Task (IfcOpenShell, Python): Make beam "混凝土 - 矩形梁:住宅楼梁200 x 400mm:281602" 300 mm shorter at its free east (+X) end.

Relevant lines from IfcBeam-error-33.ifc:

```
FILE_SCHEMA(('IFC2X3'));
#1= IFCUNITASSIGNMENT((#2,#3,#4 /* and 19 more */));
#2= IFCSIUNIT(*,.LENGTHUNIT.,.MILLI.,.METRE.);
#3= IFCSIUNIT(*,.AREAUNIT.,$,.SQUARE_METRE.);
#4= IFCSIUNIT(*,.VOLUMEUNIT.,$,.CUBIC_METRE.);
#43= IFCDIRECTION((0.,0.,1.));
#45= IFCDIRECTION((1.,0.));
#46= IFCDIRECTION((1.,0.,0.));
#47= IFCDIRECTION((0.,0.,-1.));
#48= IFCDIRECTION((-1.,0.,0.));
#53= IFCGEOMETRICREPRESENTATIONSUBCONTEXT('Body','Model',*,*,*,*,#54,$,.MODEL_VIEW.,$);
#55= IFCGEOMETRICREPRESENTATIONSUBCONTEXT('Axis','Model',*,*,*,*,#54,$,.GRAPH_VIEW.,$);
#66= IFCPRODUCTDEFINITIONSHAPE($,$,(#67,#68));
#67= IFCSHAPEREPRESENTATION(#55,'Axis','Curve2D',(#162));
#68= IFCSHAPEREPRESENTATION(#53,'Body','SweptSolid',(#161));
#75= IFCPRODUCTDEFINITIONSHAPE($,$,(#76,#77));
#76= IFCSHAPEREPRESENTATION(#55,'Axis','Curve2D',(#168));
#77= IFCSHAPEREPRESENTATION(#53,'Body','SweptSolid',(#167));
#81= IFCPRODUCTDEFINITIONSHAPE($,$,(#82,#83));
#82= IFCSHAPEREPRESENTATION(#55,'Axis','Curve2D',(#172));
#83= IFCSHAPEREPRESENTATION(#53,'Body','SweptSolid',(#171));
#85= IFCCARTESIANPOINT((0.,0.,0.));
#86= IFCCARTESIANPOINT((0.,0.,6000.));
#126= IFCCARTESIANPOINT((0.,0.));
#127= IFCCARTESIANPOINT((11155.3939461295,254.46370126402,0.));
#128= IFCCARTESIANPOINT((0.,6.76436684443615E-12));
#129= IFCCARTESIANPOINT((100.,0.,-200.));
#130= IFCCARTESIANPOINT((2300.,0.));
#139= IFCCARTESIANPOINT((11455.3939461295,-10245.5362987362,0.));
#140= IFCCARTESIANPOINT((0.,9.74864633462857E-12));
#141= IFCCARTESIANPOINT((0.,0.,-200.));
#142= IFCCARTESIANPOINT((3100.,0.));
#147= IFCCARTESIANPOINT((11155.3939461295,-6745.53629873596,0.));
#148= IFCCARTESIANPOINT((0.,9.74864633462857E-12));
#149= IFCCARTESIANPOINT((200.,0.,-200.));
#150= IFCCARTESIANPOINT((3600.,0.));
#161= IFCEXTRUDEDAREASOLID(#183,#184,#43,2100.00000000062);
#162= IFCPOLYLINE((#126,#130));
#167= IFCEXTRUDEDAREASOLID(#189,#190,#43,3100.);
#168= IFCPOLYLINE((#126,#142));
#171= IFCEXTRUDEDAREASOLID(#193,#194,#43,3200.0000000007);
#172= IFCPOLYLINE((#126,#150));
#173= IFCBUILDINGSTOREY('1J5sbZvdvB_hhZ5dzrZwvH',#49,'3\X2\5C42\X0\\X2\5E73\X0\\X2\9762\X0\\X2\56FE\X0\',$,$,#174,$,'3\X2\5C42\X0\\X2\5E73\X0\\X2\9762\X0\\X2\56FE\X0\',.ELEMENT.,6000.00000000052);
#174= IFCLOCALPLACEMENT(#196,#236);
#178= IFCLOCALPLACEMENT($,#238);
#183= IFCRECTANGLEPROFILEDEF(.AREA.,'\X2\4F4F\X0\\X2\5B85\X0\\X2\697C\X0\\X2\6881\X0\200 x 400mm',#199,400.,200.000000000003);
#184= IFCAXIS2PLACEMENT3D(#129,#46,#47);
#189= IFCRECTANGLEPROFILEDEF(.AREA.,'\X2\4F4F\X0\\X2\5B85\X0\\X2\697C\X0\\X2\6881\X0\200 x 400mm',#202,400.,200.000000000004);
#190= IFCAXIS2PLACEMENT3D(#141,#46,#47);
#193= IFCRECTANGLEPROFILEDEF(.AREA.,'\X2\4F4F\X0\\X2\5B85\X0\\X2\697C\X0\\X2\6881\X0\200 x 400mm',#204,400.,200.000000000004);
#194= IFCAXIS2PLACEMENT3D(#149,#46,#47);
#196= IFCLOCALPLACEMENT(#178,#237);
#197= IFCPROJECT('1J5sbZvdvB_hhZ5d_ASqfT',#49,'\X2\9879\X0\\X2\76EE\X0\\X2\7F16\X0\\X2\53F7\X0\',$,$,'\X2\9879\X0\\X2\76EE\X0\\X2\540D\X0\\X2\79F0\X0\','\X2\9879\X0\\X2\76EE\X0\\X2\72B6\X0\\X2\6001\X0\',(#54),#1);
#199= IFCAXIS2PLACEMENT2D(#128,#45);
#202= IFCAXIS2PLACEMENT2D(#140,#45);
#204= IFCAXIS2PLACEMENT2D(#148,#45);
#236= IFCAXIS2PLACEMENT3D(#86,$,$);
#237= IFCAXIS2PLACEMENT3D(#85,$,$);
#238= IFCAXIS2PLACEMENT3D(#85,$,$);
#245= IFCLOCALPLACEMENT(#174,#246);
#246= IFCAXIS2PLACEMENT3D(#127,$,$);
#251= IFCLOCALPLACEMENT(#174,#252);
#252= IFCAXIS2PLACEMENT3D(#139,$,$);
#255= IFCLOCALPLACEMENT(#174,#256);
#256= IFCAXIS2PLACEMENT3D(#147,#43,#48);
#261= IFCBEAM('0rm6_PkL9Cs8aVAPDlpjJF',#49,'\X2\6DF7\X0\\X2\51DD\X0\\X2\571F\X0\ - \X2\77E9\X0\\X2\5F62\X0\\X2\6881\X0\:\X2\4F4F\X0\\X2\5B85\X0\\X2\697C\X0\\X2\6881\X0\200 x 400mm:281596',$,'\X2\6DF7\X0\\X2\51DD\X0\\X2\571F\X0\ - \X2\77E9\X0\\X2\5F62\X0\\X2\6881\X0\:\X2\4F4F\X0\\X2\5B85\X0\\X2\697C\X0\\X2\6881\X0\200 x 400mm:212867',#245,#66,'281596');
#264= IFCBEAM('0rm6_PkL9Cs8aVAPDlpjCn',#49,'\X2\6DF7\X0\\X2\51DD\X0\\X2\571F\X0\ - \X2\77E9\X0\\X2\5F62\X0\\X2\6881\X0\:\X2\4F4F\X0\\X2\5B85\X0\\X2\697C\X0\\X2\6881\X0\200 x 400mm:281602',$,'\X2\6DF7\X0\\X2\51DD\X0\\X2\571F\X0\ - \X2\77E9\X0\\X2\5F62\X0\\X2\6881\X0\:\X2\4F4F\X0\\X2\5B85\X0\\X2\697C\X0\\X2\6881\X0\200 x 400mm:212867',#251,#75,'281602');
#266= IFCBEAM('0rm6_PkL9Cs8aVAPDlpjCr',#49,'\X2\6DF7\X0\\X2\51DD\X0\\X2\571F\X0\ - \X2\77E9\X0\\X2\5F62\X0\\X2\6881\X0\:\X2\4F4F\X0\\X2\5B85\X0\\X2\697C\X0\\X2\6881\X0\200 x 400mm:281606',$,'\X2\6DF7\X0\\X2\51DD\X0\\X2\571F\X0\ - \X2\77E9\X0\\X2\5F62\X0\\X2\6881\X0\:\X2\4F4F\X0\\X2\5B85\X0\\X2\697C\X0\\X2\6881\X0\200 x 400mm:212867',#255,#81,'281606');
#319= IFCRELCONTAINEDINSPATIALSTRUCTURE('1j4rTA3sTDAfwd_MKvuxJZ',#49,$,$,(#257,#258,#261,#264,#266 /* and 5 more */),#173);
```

```python
import numpy as np
import ifcopenshell
import ifcopenshell.util.representation
import ifcopenshell.util.unit

model = ifcopenshell.open("IfcBeam-error-33.ifc")
unit_scale = ifcopenshell.util.unit.calculate_unit_scale(model)

member = model.by_guid("0rm6_PkL9Cs8aVAPDlpjCn")
change = -0.3 / unit_scale

# The extrusion runs towards the end named, so only its depth changes.
body = ifcopenshell.util.representation.get_representation(member, "Model", "Body")
solid = body.Items[0]
old_length = solid.Depth
solid.Depth += change

# Move the axis end point with it.
axis = next(r for r in member.Representation.Representations if r.RepresentationIdentifier == "Axis").Items[0]
start, end = (np.array(p.Coordinates) for p in axis.Points)
end = end + (end - start) / np.linalg.norm(end - start) * change
point = model.createIfcCartesianPoint(end.tolist())
axis.Points = [axis.Points[0], point]

print(f"length {old_length:g} -> {solid.Depth:g}")

model.write("IfcBeam-error-33_rev.ifc")
```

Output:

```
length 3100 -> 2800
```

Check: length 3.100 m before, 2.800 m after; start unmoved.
